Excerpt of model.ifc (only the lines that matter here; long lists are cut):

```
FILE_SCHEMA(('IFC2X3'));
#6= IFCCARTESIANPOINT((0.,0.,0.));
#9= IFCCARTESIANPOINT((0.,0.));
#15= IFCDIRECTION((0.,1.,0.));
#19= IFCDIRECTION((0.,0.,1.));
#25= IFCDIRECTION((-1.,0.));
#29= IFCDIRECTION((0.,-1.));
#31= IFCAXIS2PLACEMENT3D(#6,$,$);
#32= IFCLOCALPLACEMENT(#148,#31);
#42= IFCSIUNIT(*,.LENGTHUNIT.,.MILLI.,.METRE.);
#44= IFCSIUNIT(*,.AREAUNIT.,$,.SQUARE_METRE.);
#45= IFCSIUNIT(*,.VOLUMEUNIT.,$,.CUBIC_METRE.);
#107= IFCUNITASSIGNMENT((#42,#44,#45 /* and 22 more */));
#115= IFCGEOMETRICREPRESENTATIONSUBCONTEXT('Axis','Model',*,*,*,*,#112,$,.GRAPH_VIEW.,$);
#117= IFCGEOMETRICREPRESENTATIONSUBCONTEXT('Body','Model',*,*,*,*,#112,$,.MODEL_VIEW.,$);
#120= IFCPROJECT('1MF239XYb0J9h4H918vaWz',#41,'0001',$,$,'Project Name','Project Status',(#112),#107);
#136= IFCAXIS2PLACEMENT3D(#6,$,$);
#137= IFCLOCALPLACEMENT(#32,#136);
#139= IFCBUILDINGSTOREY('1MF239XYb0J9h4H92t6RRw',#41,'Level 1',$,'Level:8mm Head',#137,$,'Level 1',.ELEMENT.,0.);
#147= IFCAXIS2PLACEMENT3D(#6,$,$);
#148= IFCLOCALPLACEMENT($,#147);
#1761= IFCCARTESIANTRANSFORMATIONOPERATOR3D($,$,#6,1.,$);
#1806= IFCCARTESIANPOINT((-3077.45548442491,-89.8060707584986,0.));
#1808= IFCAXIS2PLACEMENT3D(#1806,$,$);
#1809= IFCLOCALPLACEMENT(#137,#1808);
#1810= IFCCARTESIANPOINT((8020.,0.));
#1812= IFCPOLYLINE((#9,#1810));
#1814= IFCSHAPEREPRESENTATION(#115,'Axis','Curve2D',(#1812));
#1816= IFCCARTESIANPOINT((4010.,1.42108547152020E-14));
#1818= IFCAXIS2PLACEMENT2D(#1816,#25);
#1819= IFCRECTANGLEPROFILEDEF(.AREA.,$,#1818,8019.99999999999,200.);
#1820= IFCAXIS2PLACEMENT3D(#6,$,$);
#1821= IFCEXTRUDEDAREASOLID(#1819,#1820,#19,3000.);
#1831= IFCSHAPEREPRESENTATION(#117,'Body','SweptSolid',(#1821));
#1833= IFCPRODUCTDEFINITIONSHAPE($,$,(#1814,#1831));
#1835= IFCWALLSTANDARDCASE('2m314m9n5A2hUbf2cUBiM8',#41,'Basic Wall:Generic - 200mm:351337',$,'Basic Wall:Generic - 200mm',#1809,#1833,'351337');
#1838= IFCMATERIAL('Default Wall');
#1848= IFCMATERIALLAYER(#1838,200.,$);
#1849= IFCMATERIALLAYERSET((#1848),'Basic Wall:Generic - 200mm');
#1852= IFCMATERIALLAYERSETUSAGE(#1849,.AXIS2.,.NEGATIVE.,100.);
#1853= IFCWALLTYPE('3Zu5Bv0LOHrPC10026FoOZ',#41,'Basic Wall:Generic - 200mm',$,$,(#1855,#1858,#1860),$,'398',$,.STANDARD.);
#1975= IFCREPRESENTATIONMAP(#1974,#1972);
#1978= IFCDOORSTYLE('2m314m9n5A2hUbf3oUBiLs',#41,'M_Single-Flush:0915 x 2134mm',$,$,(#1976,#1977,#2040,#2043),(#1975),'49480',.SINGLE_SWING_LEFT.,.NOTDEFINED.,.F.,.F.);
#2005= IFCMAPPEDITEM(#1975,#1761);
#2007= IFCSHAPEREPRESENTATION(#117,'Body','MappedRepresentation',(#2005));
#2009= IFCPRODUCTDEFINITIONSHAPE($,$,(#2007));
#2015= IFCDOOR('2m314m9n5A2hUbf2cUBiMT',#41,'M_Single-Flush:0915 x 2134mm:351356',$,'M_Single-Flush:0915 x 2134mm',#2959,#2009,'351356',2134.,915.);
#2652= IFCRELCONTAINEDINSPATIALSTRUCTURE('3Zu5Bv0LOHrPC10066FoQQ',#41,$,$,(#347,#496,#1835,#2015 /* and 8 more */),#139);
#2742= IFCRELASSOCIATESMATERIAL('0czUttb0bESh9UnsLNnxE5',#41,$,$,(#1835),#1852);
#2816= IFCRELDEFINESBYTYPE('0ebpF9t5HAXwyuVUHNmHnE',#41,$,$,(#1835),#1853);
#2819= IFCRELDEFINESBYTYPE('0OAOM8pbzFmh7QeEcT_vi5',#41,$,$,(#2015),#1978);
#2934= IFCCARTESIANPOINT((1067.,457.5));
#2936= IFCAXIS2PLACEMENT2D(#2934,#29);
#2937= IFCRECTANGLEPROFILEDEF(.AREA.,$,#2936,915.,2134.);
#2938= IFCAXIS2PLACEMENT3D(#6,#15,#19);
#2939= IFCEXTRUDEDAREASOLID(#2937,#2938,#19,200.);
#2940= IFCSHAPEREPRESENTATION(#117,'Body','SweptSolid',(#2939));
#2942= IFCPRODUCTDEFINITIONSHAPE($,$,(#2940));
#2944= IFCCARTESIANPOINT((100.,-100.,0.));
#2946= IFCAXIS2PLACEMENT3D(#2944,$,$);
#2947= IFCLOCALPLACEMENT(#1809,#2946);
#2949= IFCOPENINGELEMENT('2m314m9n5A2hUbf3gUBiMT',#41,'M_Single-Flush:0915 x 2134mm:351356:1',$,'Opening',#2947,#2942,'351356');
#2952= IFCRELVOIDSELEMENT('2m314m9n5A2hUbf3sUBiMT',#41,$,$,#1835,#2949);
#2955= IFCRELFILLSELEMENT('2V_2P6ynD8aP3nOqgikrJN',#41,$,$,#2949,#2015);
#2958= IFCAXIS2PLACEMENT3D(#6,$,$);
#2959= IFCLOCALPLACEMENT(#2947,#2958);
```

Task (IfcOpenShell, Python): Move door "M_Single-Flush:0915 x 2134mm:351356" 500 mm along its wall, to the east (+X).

```python
import ifcopenshell
import ifcopenshell.api.geometry
import ifcopenshell.util.placement

model = ifcopenshell.open("model.ifc")

door = model.by_guid("2m314m9n5A2hUbf2cUBiMT")
opening = door.FillsVoids[0].RelatingOpeningElement
wall = opening.VoidsElements[0].RelatingBuildingElement

wall_matrix = ifcopenshell.util.placement.get_local_placement(wall.ObjectPlacement)
shift = wall_matrix[:3, 0] * 500.0
before = ifcopenshell.util.placement.get_local_placement(door.ObjectPlacement)[:3, 3].copy()

# The door is placed relative to its opening, so it follows when the opening moves.
matrix = ifcopenshell.util.placement.get_local_placement(opening.ObjectPlacement)
matrix[:3, 3] += shift
ifcopenshell.api.geometry.edit_object_placement(
    model, product=opening, matrix=matrix, is_si=False, should_transform_children=True
)

after = ifcopenshell.util.placement.get_local_placement(door.ObjectPlacement)[:3, 3]
print("door moved by", (after - before).round(3) + 0.0)

model.write("model_v2.ifc")
```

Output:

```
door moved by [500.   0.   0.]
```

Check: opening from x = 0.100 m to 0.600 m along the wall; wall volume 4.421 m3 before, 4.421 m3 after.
